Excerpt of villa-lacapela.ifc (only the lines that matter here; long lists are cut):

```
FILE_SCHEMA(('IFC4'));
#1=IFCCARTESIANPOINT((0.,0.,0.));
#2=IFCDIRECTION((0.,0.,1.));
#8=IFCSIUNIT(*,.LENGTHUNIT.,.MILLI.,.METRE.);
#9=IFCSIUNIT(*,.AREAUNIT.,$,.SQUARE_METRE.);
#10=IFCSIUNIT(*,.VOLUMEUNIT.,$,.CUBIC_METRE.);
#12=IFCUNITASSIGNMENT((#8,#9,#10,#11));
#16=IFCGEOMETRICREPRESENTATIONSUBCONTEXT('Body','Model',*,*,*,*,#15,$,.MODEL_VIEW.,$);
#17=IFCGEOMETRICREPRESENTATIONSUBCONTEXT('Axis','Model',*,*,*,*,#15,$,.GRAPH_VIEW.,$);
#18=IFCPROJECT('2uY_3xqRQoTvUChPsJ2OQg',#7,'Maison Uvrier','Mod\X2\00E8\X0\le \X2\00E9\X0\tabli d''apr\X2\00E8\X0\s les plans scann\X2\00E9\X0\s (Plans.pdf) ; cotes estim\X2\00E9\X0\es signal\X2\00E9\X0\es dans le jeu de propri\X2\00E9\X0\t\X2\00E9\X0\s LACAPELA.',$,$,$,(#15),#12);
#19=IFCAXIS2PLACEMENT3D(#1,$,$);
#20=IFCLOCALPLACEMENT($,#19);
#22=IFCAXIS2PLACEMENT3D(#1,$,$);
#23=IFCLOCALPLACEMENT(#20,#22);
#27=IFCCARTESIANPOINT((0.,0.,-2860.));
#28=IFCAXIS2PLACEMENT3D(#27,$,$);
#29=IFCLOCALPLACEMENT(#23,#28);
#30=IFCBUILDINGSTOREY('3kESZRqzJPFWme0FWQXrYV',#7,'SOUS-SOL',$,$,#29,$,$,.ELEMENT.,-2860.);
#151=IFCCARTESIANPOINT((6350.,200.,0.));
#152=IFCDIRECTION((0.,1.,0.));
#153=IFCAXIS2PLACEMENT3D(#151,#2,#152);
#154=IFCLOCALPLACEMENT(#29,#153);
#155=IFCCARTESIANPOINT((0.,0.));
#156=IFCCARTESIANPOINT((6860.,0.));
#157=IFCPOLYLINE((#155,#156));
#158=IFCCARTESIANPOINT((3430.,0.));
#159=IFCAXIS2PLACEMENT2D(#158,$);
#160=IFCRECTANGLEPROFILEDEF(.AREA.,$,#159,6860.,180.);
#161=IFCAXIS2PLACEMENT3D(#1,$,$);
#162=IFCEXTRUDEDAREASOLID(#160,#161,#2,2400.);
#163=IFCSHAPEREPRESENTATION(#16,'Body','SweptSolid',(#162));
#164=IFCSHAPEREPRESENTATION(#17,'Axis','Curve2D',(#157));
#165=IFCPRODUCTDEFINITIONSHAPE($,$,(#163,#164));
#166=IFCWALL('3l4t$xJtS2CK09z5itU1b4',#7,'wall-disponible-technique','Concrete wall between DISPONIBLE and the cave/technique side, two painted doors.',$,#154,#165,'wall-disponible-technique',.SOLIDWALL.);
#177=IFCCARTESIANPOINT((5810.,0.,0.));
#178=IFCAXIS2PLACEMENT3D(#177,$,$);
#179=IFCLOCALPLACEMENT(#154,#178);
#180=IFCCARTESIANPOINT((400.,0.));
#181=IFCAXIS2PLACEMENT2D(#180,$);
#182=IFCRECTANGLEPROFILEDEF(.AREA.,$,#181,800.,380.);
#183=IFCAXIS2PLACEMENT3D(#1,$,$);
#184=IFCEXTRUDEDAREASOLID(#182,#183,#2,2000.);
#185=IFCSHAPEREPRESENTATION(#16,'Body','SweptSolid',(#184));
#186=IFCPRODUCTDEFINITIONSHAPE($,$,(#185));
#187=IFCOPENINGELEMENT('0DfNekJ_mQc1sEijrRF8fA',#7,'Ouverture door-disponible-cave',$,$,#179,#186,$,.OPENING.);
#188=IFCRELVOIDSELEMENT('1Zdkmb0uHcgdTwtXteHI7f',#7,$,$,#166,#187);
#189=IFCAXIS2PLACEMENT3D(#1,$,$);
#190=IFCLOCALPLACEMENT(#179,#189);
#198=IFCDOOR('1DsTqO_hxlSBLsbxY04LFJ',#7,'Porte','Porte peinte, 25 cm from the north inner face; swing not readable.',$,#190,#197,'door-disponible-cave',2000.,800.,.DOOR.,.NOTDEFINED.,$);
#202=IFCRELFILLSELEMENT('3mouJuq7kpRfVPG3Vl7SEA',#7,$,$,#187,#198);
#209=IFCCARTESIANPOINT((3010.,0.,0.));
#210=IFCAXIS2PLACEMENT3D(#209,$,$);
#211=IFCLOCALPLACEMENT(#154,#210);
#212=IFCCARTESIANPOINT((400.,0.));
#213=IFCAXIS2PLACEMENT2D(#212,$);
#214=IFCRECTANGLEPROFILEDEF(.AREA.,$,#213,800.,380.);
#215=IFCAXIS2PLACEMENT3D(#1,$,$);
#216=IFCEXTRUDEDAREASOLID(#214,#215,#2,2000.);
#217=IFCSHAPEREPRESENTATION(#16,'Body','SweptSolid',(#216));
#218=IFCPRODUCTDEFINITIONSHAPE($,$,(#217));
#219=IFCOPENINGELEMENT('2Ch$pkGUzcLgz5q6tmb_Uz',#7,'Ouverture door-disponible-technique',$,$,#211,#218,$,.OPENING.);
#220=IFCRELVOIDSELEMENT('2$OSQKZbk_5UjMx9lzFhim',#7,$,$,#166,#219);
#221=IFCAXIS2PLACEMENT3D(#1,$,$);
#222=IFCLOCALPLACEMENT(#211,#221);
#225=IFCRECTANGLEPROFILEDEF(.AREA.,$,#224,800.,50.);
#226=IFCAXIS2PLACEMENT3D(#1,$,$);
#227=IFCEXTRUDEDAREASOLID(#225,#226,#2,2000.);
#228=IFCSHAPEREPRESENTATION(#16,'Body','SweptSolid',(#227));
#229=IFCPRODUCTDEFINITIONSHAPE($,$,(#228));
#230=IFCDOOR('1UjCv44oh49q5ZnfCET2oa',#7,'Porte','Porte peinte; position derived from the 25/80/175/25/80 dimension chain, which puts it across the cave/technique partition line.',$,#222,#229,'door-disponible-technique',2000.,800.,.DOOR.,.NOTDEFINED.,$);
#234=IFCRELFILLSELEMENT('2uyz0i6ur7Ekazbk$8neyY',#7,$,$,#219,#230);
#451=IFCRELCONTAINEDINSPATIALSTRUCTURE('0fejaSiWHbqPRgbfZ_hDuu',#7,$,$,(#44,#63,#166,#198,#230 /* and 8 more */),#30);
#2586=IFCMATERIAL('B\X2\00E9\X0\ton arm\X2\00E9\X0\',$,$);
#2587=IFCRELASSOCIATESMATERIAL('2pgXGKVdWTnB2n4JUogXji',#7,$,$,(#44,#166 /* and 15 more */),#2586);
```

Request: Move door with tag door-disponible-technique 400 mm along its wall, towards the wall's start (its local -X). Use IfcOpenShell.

```python
import ifcopenshell
import ifcopenshell.api.geometry
import ifcopenshell.util.placement

model = ifcopenshell.open("villa-lacapela.ifc")

door = model.by_guid("1UjCv44oh49q5ZnfCET2oa")
opening = door.FillsVoids[0].RelatingOpeningElement
wall = opening.VoidsElements[0].RelatingBuildingElement

wall_matrix = ifcopenshell.util.placement.get_local_placement(wall.ObjectPlacement)
shift = wall_matrix[:3, 0] * -400.0
before = ifcopenshell.util.placement.get_local_placement(door.ObjectPlacement)[:3, 3].copy()

# The door is placed relative to its opening, so it follows when the opening moves.
matrix = ifcopenshell.util.placement.get_local_placement(opening.ObjectPlacement)
matrix[:3, 3] += shift
ifcopenshell.api.geometry.edit_object_placement(
    model, product=opening, matrix=matrix, is_si=False, should_transform_children=True
)

after = ifcopenshell.util.placement.get_local_placement(door.ObjectPlacement)[:3, 3]
print("door moved by", (after - before).round(3) + 0.0)

model.write("villa-lacapela_rev.ifc")
```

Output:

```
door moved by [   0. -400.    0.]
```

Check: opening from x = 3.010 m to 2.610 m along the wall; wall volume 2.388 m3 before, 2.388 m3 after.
